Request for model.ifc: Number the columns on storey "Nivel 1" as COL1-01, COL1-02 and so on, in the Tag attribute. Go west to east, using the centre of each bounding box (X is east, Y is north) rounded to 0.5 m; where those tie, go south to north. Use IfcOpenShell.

First a look at what the model holds.

```python
import ifcopenshell
import ifcopenshell.util.element
import ifcopenshell.util.placement

model = ifcopenshell.open("model.ifc")
print(model.schema)
storey = next(s for s in model.by_type("IfcBuildingStorey") if s.Name == "Nivel 1")
columns = [e for e in ifcopenshell.util.element.get_decomposition(storey) if e.is_a("IfcColumn")]
for e in sorted(columns, key=lambda e: e.id()):
    origin = ifcopenshell.util.placement.get_local_placement(e.ObjectPlacement)[:3, 3]
    print(e.id(), e.Tag, e.Name, origin.round(2) + 0.0, sep=" | ")
```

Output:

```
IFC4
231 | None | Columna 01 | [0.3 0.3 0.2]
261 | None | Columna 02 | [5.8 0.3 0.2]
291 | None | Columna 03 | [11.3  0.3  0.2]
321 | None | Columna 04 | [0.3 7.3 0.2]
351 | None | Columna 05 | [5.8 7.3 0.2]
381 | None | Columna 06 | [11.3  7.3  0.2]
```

```python
import ifcopenshell
import ifcopenshell.geom
import ifcopenshell.util.element
import ifcopenshell.util.shape

model = ifcopenshell.open("model.ifc")
settings = ifcopenshell.geom.settings()
settings.set("use-world-coords", True)


def centre(element):
    shape = ifcopenshell.geom.create_shape(settings, element)
    return ifcopenshell.util.shape.get_bbox_centroid(shape.geometry)


storey = next(s for s in model.by_type("IfcBuildingStorey") if s.Name == "Nivel 1")
columns = [e for e in ifcopenshell.util.element.get_decomposition(storey) if e.is_a("IfcColumn")]

# Insertion points can sit at a corner or the storey origin, so sort by the geometry (in metres).
centres = {e: centre(e) for e in columns}
columns.sort(key=lambda e: (round(centres[e][0] / 0.5), centres[e][1]))

for i, e in enumerate(columns, start=1):
    number = f"COL1-{i:02d}"
    e.Tag = number
    print(e.id(), number)

model.write("model_v2.ifc")
```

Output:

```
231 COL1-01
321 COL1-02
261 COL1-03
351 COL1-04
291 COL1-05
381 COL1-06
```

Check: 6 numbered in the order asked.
